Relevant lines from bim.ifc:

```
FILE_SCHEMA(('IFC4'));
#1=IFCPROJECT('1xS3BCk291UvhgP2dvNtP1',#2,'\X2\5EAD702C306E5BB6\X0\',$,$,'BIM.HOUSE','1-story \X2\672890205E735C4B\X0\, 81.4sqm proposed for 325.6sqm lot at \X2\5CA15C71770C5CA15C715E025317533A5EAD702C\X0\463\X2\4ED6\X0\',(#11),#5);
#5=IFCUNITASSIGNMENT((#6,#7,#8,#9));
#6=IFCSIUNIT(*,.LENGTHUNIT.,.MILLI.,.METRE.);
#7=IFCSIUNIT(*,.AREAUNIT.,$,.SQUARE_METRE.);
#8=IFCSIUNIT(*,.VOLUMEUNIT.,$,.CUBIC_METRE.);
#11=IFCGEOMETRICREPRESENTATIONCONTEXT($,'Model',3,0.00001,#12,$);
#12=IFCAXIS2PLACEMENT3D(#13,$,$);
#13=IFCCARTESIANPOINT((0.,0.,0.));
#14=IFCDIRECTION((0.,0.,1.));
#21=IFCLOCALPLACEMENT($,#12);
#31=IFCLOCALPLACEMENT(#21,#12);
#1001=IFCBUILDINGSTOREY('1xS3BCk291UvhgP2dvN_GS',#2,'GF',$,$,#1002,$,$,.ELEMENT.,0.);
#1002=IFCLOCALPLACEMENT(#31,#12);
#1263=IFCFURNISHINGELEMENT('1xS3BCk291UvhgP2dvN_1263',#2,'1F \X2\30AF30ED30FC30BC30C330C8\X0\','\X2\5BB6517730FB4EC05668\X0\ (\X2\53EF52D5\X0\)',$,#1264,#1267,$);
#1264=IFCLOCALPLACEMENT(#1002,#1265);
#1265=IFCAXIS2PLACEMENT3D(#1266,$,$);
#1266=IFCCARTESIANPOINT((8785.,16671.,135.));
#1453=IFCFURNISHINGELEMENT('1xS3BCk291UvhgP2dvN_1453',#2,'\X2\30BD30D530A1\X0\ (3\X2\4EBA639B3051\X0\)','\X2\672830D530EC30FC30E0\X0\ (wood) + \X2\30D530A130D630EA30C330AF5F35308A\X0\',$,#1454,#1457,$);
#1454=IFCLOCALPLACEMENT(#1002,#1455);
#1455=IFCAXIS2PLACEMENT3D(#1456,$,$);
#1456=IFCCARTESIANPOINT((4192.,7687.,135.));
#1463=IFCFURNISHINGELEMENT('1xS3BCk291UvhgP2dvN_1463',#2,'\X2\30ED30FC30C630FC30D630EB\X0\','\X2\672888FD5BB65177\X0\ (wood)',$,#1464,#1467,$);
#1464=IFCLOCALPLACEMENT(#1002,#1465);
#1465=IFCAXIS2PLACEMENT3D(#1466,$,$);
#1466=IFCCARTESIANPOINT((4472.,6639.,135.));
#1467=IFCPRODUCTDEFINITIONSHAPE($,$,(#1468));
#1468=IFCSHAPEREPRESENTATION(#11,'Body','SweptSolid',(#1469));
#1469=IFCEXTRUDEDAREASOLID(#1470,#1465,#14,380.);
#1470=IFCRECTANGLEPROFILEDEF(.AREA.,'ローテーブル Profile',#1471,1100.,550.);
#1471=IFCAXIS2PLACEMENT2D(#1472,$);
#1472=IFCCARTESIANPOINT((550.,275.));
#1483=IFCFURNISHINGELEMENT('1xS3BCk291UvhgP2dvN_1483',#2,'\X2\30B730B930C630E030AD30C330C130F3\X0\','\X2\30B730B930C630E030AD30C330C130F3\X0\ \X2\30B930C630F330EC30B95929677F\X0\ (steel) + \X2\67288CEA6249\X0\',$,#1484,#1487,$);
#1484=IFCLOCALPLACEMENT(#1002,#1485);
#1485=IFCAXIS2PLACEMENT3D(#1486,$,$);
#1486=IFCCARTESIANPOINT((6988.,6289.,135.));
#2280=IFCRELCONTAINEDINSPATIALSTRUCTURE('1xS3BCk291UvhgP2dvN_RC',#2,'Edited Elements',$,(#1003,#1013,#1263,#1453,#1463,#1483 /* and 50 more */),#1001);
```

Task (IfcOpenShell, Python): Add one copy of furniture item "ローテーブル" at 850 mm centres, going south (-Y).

```python
import numpy as np
import ifcopenshell
import ifcopenshell.api.geometry
import ifcopenshell.api.root
import ifcopenshell.util.element
import ifcopenshell.util.placement
import ifcopenshell.util.unit

model = ifcopenshell.open("bim.ifc")
unit_scale = ifcopenshell.util.unit.calculate_unit_scale(model)


def reuse_history(source, copy):
    """copy_class also copies each property set's owner history, people and application; keep the originals."""
    for rel in copy.IsDefinedBy:
        if rel.is_a("IfcRelDefinesByProperties") and (history := rel.RelatingPropertyDefinition.OwnerHistory):
            rel.RelatingPropertyDefinition.OwnerHistory = source.OwnerHistory
            ifcopenshell.util.element.remove_deep2(model, history)


source = model.by_guid("1xS3BCk291UvhgP2dvN_1463")
base = ifcopenshell.util.placement.get_local_placement(source.ObjectPlacement)
step = np.array([0.0, -1.0, 0.0]) * 0.85 / unit_scale

for i in range(1, 2):
    copy = ifcopenshell.api.root.copy_class(model, product=source)
    copy.Representation = ifcopenshell.util.element.copy_deep(
        model, source.Representation, exclude=["IfcGeometricRepresentationContext", "IfcRepresentationMap"]
    )
    reuse_history(source, copy)
    matrix = base.copy()
    matrix[:3, 3] += i * step
    print("added at", matrix[:3, 3].round(3) + 0.0)
    ifcopenshell.api.geometry.edit_object_placement(model, product=copy, matrix=matrix, is_si=False)

model.write("bim_edited.ifc")
```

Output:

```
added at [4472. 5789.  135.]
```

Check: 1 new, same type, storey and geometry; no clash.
